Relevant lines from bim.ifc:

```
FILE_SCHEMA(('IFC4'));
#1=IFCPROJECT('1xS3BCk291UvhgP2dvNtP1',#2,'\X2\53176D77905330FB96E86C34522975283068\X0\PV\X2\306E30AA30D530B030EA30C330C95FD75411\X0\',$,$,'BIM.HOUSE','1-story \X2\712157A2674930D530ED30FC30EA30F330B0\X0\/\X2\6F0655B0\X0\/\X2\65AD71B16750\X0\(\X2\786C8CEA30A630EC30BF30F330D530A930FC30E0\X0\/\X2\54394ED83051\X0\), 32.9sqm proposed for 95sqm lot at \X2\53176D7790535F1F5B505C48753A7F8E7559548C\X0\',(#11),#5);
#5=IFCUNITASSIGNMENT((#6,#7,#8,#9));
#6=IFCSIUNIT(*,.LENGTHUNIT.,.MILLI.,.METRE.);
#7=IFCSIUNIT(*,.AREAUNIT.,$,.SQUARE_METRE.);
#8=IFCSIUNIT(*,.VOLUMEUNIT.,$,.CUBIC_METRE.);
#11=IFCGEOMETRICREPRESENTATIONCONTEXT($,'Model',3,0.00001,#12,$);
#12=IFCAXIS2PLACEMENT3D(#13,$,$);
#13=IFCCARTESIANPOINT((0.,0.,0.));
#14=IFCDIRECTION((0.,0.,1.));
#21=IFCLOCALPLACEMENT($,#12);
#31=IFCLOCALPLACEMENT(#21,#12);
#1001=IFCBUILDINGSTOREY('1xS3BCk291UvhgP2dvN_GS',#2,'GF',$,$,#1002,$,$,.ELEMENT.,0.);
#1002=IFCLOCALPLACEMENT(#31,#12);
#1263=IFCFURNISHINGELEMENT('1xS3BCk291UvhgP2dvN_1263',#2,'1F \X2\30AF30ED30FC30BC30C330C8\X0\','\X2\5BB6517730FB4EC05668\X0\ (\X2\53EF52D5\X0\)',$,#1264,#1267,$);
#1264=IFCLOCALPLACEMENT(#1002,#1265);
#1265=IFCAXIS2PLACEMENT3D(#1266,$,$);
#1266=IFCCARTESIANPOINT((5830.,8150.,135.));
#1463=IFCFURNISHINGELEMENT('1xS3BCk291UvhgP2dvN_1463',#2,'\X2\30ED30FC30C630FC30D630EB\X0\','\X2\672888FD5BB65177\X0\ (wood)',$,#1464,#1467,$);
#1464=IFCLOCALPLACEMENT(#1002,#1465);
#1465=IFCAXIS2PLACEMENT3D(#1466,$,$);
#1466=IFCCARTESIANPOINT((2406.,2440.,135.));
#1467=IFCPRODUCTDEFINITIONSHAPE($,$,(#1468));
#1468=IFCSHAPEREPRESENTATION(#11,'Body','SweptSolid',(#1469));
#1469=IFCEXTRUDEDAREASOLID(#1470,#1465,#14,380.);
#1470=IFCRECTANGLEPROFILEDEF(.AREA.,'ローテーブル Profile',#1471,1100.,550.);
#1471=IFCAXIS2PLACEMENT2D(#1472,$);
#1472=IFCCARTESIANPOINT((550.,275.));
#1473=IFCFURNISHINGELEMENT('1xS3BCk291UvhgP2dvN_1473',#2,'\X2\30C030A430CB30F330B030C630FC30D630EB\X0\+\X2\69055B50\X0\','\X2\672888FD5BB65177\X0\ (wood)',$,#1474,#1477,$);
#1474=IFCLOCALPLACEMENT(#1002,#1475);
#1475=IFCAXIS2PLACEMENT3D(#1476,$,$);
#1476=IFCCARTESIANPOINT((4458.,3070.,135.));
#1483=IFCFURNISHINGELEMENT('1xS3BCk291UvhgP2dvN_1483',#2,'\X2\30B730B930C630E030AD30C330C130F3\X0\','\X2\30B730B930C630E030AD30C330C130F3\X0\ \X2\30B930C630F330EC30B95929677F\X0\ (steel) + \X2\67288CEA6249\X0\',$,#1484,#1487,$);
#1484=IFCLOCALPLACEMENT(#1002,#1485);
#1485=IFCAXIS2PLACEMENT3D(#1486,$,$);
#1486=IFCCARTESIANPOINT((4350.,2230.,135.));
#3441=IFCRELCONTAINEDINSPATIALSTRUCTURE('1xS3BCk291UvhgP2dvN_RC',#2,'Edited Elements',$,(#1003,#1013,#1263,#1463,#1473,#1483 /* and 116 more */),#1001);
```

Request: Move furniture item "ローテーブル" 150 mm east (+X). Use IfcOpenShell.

```python
import ifcopenshell
import ifcopenshell.api.geometry
import ifcopenshell.util.placement

model = ifcopenshell.open("bim.ifc")

item = model.by_guid("1xS3BCk291UvhgP2dvN_1463")
matrix = ifcopenshell.util.placement.get_local_placement(item.ObjectPlacement)
matrix[0, 3] += 150.0
ifcopenshell.api.geometry.edit_object_placement(model, product=item, matrix=matrix, is_si=False)

print(ifcopenshell.util.placement.get_local_placement(item.ObjectPlacement).round(3) + 0.0)

model.write("bim_rev.ifc")
```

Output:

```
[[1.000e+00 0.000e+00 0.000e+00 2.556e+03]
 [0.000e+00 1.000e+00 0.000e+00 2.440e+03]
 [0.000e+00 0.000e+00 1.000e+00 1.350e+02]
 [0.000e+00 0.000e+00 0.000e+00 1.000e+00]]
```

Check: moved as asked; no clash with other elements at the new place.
